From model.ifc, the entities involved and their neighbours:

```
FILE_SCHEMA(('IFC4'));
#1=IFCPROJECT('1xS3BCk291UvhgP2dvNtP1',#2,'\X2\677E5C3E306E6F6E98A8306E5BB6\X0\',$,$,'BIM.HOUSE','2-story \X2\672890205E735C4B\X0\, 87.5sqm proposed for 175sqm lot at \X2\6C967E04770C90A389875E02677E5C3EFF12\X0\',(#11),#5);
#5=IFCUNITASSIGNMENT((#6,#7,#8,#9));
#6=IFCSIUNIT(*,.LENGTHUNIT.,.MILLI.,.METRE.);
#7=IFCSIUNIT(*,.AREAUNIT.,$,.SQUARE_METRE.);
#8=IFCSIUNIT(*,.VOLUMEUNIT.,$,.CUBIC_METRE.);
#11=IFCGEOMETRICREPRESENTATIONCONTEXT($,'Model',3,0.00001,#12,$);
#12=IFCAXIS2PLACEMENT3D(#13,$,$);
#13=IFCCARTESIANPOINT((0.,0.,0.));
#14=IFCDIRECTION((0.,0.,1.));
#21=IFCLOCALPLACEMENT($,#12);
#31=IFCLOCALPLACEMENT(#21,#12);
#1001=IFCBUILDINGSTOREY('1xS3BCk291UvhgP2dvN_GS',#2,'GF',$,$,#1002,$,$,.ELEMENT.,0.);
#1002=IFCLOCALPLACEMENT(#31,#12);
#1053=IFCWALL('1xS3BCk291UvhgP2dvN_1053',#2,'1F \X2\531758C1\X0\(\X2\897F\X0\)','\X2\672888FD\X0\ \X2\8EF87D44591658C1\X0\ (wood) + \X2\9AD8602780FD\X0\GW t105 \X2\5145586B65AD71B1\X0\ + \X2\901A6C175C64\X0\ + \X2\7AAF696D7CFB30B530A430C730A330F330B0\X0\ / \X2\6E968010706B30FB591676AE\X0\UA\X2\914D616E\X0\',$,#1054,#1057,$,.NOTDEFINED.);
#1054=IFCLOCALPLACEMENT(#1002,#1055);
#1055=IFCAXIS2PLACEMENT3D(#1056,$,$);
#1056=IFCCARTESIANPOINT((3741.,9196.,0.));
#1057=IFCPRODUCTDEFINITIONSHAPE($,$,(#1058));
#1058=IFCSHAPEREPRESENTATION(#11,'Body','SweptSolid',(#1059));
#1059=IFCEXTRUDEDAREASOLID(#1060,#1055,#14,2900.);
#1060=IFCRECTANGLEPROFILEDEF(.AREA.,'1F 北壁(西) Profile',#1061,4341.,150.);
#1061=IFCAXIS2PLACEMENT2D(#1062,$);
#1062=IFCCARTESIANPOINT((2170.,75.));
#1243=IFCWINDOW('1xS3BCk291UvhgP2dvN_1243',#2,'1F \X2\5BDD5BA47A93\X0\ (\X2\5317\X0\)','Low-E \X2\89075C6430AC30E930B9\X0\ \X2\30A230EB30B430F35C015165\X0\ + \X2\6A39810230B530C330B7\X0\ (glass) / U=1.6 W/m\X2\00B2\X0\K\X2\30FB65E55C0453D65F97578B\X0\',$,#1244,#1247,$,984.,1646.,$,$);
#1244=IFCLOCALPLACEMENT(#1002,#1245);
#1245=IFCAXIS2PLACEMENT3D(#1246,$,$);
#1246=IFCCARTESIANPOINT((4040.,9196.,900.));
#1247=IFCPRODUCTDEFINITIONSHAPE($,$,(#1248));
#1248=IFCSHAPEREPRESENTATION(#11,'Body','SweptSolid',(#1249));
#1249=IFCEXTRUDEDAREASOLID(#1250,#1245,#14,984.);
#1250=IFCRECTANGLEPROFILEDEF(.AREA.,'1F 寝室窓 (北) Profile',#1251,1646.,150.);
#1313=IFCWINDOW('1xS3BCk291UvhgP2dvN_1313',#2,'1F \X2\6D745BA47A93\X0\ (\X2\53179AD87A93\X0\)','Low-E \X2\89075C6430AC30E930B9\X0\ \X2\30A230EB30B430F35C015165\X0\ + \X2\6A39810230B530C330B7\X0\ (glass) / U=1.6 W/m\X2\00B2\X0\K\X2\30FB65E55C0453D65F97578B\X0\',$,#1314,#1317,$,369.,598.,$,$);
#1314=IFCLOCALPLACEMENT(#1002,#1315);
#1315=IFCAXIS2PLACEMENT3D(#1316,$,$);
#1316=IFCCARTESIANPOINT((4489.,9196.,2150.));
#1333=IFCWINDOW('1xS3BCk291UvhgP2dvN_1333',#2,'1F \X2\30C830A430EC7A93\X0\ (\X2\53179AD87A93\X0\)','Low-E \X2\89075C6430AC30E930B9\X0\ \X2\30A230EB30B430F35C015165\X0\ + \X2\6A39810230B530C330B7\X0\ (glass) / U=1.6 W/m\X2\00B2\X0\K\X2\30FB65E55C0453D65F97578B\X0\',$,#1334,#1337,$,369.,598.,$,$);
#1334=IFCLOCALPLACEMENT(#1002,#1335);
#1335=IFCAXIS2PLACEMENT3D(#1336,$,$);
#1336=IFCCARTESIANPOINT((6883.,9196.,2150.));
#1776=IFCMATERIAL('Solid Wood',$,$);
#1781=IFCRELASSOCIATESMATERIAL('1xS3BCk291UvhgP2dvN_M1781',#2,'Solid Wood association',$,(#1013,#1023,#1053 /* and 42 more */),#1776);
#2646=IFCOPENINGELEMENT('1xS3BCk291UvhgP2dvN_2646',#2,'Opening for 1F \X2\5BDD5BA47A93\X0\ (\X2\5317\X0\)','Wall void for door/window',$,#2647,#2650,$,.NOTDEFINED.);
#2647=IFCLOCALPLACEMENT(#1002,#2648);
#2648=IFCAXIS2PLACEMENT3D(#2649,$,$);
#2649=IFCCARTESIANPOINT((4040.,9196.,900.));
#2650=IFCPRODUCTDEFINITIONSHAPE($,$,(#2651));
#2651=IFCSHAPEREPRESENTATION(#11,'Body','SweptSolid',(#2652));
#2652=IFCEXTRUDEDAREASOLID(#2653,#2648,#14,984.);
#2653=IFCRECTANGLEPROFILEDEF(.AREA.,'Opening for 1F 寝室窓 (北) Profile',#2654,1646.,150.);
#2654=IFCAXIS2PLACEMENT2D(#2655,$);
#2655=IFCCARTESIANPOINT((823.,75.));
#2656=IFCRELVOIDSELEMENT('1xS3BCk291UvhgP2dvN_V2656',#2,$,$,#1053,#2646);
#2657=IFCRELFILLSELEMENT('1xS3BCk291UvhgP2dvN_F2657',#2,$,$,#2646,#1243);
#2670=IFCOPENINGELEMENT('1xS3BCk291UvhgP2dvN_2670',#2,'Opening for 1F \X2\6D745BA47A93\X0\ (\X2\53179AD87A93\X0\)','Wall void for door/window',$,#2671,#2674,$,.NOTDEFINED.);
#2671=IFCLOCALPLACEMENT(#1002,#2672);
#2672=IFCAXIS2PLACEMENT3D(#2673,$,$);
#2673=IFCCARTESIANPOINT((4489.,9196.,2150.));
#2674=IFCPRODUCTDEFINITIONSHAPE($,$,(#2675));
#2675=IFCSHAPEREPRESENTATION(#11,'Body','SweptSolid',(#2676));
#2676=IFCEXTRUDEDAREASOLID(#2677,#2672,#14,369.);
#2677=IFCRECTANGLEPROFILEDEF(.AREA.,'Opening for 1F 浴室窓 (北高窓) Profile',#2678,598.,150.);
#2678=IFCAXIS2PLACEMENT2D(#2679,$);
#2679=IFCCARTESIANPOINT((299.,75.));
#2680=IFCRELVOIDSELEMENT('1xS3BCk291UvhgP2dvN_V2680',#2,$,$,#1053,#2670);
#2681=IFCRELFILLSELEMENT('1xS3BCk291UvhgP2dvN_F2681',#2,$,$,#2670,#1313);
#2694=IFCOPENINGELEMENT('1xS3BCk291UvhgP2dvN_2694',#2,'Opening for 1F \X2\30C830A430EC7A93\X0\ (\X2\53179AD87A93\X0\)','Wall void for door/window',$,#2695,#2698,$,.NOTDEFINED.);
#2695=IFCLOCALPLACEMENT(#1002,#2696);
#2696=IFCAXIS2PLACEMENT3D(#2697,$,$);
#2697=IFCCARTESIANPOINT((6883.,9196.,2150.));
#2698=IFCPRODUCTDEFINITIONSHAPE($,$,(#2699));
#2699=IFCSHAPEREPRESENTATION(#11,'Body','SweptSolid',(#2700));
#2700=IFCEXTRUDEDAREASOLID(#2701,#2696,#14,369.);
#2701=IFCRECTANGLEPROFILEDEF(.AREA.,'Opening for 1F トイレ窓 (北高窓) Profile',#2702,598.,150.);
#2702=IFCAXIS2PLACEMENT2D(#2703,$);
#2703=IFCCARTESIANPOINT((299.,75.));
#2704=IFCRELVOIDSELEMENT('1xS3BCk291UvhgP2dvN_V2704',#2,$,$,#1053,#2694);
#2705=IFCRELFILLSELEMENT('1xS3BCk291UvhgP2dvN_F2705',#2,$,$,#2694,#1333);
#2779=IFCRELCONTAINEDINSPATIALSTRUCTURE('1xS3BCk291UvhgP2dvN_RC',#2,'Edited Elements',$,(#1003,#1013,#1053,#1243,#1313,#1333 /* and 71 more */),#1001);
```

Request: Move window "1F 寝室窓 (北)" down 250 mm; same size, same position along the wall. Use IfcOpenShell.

```python
import numpy as np
import ifcopenshell
import ifcopenshell.api.geometry
import ifcopenshell.util.placement
import ifcopenshell.util.unit

model = ifcopenshell.open("model.ifc")
unit_scale = ifcopenshell.util.unit.calculate_unit_scale(model)

window = model.by_id(1243)
opening = window.FillsVoids[0].RelatingOpeningElement
dz = -250.0

shift = np.array([0.0, 0.0, dz])
# The window is not placed relative to its opening, so move both.
for product in (opening, window):
    matrix = ifcopenshell.util.placement.get_local_placement(product.ObjectPlacement)
    matrix[:3, 3] += shift
    ifcopenshell.api.geometry.edit_object_placement(model, product=product, matrix=matrix, is_si=False)

print(f"moved by {dz * unit_scale:+.3f} m")

model.write("model-out.ifc")
```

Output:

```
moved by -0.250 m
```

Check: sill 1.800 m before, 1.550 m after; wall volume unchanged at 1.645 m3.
